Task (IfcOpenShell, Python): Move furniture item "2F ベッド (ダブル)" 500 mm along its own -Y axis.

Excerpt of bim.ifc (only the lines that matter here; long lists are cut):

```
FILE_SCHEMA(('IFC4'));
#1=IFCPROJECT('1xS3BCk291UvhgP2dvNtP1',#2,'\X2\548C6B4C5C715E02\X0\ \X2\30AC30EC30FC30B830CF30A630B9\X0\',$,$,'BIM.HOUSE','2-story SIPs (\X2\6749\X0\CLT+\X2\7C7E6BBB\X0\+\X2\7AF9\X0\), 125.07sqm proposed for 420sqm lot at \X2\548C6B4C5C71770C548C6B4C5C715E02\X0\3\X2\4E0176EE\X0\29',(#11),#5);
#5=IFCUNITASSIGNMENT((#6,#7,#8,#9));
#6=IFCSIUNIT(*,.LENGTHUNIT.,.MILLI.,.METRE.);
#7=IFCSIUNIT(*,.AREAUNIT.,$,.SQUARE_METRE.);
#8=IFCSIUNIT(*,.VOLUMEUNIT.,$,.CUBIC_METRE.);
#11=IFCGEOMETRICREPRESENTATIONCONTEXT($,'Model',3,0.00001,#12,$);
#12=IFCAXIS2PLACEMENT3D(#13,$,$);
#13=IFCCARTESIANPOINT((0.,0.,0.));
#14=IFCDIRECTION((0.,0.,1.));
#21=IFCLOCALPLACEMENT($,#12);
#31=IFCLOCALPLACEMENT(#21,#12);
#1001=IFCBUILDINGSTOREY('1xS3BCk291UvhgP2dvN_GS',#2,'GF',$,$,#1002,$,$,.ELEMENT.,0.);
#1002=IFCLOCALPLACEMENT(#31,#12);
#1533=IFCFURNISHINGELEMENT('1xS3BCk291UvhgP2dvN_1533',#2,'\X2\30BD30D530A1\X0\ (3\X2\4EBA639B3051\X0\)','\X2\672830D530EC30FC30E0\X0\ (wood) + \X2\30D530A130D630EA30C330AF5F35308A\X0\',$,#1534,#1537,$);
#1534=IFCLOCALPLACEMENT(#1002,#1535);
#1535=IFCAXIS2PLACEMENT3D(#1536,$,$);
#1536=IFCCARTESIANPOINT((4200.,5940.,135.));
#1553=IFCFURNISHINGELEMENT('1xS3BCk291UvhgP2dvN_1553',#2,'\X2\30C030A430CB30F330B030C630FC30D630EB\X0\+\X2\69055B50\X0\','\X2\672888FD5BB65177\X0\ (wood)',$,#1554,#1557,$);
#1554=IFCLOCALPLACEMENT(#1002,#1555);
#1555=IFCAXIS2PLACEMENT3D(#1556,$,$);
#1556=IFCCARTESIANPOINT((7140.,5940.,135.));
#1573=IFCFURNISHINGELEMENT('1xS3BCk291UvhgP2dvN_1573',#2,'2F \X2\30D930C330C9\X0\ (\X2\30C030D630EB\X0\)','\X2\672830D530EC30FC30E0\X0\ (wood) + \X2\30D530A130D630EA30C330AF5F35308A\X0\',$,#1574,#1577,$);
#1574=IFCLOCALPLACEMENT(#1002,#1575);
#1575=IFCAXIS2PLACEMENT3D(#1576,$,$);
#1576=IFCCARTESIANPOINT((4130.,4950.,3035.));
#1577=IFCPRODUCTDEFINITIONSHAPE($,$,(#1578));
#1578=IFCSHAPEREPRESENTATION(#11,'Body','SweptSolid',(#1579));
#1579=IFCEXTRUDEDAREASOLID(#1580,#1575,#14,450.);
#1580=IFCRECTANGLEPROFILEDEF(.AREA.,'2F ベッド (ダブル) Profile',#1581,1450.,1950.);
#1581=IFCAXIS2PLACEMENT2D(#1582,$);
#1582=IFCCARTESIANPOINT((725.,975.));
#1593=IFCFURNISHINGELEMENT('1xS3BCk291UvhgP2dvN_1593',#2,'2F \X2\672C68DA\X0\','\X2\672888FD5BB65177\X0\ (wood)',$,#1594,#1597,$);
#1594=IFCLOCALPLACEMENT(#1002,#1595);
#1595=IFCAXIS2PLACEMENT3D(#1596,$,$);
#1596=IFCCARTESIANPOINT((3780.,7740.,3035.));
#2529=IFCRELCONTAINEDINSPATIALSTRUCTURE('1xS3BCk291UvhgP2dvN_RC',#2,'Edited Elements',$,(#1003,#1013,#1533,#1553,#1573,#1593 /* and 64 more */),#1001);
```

```python
import ifcopenshell
import ifcopenshell.api.geometry
import ifcopenshell.util.placement

model = ifcopenshell.open("bim.ifc")

item = model.by_guid("1xS3BCk291UvhgP2dvN_1573")
matrix = ifcopenshell.util.placement.get_local_placement(item.ObjectPlacement)
matrix[:3, 3] -= matrix[:3, 1] * 500.0
ifcopenshell.api.geometry.edit_object_placement(model, product=item, matrix=matrix, is_si=False)

print(ifcopenshell.util.placement.get_local_placement(item.ObjectPlacement).round(3) + 0.0)

model.write("bim_updated.ifc")
```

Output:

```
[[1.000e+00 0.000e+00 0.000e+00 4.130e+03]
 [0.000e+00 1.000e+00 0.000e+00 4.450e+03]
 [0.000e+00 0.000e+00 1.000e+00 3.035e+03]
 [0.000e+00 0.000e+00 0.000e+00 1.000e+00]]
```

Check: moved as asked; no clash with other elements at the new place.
